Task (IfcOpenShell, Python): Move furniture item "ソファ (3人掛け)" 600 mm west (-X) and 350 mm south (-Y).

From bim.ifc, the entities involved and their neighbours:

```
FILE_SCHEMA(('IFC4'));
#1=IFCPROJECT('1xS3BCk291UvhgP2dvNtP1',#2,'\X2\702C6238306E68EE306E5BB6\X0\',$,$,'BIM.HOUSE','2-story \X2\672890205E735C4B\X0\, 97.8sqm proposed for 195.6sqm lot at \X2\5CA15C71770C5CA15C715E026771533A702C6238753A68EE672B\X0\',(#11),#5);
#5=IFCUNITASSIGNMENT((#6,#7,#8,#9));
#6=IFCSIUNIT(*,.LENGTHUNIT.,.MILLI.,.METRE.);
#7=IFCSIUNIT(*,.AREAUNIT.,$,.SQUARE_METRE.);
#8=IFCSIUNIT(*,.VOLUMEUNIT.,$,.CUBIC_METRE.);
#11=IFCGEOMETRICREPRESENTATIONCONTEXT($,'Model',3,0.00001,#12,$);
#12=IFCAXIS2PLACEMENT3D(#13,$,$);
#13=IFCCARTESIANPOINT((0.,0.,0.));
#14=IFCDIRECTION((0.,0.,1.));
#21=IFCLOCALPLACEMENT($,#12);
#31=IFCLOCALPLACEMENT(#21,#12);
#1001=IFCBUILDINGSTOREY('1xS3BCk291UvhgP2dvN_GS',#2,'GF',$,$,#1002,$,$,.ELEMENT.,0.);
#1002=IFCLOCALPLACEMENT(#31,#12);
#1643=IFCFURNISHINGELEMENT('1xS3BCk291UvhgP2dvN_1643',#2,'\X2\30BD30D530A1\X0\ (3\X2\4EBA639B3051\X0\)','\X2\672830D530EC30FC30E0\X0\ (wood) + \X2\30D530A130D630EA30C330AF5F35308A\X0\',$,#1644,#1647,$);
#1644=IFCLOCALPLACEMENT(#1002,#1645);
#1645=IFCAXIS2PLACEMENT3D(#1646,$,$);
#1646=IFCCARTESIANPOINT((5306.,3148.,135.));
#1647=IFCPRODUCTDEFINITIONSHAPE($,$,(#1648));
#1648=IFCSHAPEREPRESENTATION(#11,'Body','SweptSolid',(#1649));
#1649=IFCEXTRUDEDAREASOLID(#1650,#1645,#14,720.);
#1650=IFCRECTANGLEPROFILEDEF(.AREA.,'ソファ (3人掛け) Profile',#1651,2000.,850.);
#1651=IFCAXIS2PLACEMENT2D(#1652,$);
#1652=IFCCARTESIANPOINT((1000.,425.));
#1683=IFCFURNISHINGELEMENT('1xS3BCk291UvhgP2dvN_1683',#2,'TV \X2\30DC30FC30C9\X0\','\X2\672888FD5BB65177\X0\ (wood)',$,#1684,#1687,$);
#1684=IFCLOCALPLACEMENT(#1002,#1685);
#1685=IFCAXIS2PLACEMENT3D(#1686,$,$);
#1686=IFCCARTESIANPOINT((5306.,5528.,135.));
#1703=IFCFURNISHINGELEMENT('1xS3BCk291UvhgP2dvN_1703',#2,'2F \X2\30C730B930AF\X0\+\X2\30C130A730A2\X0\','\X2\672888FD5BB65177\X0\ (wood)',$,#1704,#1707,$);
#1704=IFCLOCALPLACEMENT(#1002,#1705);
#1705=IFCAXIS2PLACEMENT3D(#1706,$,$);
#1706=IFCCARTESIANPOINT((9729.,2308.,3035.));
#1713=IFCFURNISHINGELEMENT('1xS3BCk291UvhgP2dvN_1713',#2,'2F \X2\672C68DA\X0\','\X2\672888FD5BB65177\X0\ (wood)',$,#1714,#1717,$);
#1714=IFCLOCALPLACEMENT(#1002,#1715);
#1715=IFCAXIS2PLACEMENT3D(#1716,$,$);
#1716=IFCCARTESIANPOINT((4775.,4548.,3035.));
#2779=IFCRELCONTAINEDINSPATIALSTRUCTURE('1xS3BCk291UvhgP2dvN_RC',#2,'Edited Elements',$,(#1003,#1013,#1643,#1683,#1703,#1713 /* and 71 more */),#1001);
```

```python
import ifcopenshell
import ifcopenshell.api.geometry
import ifcopenshell.util.placement
import ifcopenshell.util.unit

model = ifcopenshell.open("bim.ifc")
unit_scale = ifcopenshell.util.unit.calculate_unit_scale(model)

item = model.by_guid("1xS3BCk291UvhgP2dvN_1643")
matrix = ifcopenshell.util.placement.get_local_placement(item.ObjectPlacement)
matrix[0, 3] -= 0.6 / unit_scale
matrix[1, 3] -= 0.35 / unit_scale
ifcopenshell.api.geometry.edit_object_placement(model, product=item, matrix=matrix, is_si=False)

print(ifcopenshell.util.placement.get_local_placement(item.ObjectPlacement).round(3) + 0.0)

model.write("bim-out.ifc")
```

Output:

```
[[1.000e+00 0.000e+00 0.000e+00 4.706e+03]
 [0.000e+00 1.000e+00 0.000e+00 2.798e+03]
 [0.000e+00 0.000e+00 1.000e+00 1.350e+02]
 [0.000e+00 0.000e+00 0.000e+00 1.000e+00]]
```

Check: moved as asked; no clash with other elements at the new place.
